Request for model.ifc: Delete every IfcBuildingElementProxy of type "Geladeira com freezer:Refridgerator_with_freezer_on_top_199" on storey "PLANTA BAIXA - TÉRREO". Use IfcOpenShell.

First a look at what the model holds.

```python
import ifcopenshell
import ifcopenshell.util.element

model = ifcopenshell.open("model.ifc")
print(model.schema)
storey = next(s for s in model.by_type("IfcBuildingStorey") if s.Name == "PLANTA BAIXA - TÉRREO")
proxies = [e for e in ifcopenshell.util.element.get_decomposition(storey) if e.is_a("IfcBuildingElementProxy")]
seen = {}
for e in proxies:
    element_type = ifcopenshell.util.element.get_type(e)
    name = element_type.Name if element_type not in (None, e) else None
    seen[name] = seen.get(name, 0) + 1
for name, count in sorted(seen.items(), key=str):
    print(count, "x", name)
```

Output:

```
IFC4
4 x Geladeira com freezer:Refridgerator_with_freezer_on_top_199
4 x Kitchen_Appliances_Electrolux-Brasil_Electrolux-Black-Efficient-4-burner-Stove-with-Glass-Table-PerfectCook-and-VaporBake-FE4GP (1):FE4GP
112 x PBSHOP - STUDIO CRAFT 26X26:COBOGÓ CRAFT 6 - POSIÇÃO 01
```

```python
import ifcopenshell
import ifcopenshell.api.root
import ifcopenshell.util.element

model = ifcopenshell.open("model.ifc")

storey = next(s for s in model.by_type("IfcBuildingStorey") if s.Name == "PLANTA BAIXA - TÉRREO")
proxies = [e for e in ifcopenshell.util.element.get_decomposition(storey) if e.is_a("IfcBuildingElementProxy")]
targets = [e for e in proxies if (t := ifcopenshell.util.element.get_type(e)) not in (None, e) and t.Name == "Geladeira com freezer:Refridgerator_with_freezer_on_top_199"]

for e in targets:
    ifcopenshell.api.root.remove_product(model, product=e)
print(len(targets), "removed")

model.write("model_rev.ifc")
```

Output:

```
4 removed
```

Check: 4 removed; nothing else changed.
